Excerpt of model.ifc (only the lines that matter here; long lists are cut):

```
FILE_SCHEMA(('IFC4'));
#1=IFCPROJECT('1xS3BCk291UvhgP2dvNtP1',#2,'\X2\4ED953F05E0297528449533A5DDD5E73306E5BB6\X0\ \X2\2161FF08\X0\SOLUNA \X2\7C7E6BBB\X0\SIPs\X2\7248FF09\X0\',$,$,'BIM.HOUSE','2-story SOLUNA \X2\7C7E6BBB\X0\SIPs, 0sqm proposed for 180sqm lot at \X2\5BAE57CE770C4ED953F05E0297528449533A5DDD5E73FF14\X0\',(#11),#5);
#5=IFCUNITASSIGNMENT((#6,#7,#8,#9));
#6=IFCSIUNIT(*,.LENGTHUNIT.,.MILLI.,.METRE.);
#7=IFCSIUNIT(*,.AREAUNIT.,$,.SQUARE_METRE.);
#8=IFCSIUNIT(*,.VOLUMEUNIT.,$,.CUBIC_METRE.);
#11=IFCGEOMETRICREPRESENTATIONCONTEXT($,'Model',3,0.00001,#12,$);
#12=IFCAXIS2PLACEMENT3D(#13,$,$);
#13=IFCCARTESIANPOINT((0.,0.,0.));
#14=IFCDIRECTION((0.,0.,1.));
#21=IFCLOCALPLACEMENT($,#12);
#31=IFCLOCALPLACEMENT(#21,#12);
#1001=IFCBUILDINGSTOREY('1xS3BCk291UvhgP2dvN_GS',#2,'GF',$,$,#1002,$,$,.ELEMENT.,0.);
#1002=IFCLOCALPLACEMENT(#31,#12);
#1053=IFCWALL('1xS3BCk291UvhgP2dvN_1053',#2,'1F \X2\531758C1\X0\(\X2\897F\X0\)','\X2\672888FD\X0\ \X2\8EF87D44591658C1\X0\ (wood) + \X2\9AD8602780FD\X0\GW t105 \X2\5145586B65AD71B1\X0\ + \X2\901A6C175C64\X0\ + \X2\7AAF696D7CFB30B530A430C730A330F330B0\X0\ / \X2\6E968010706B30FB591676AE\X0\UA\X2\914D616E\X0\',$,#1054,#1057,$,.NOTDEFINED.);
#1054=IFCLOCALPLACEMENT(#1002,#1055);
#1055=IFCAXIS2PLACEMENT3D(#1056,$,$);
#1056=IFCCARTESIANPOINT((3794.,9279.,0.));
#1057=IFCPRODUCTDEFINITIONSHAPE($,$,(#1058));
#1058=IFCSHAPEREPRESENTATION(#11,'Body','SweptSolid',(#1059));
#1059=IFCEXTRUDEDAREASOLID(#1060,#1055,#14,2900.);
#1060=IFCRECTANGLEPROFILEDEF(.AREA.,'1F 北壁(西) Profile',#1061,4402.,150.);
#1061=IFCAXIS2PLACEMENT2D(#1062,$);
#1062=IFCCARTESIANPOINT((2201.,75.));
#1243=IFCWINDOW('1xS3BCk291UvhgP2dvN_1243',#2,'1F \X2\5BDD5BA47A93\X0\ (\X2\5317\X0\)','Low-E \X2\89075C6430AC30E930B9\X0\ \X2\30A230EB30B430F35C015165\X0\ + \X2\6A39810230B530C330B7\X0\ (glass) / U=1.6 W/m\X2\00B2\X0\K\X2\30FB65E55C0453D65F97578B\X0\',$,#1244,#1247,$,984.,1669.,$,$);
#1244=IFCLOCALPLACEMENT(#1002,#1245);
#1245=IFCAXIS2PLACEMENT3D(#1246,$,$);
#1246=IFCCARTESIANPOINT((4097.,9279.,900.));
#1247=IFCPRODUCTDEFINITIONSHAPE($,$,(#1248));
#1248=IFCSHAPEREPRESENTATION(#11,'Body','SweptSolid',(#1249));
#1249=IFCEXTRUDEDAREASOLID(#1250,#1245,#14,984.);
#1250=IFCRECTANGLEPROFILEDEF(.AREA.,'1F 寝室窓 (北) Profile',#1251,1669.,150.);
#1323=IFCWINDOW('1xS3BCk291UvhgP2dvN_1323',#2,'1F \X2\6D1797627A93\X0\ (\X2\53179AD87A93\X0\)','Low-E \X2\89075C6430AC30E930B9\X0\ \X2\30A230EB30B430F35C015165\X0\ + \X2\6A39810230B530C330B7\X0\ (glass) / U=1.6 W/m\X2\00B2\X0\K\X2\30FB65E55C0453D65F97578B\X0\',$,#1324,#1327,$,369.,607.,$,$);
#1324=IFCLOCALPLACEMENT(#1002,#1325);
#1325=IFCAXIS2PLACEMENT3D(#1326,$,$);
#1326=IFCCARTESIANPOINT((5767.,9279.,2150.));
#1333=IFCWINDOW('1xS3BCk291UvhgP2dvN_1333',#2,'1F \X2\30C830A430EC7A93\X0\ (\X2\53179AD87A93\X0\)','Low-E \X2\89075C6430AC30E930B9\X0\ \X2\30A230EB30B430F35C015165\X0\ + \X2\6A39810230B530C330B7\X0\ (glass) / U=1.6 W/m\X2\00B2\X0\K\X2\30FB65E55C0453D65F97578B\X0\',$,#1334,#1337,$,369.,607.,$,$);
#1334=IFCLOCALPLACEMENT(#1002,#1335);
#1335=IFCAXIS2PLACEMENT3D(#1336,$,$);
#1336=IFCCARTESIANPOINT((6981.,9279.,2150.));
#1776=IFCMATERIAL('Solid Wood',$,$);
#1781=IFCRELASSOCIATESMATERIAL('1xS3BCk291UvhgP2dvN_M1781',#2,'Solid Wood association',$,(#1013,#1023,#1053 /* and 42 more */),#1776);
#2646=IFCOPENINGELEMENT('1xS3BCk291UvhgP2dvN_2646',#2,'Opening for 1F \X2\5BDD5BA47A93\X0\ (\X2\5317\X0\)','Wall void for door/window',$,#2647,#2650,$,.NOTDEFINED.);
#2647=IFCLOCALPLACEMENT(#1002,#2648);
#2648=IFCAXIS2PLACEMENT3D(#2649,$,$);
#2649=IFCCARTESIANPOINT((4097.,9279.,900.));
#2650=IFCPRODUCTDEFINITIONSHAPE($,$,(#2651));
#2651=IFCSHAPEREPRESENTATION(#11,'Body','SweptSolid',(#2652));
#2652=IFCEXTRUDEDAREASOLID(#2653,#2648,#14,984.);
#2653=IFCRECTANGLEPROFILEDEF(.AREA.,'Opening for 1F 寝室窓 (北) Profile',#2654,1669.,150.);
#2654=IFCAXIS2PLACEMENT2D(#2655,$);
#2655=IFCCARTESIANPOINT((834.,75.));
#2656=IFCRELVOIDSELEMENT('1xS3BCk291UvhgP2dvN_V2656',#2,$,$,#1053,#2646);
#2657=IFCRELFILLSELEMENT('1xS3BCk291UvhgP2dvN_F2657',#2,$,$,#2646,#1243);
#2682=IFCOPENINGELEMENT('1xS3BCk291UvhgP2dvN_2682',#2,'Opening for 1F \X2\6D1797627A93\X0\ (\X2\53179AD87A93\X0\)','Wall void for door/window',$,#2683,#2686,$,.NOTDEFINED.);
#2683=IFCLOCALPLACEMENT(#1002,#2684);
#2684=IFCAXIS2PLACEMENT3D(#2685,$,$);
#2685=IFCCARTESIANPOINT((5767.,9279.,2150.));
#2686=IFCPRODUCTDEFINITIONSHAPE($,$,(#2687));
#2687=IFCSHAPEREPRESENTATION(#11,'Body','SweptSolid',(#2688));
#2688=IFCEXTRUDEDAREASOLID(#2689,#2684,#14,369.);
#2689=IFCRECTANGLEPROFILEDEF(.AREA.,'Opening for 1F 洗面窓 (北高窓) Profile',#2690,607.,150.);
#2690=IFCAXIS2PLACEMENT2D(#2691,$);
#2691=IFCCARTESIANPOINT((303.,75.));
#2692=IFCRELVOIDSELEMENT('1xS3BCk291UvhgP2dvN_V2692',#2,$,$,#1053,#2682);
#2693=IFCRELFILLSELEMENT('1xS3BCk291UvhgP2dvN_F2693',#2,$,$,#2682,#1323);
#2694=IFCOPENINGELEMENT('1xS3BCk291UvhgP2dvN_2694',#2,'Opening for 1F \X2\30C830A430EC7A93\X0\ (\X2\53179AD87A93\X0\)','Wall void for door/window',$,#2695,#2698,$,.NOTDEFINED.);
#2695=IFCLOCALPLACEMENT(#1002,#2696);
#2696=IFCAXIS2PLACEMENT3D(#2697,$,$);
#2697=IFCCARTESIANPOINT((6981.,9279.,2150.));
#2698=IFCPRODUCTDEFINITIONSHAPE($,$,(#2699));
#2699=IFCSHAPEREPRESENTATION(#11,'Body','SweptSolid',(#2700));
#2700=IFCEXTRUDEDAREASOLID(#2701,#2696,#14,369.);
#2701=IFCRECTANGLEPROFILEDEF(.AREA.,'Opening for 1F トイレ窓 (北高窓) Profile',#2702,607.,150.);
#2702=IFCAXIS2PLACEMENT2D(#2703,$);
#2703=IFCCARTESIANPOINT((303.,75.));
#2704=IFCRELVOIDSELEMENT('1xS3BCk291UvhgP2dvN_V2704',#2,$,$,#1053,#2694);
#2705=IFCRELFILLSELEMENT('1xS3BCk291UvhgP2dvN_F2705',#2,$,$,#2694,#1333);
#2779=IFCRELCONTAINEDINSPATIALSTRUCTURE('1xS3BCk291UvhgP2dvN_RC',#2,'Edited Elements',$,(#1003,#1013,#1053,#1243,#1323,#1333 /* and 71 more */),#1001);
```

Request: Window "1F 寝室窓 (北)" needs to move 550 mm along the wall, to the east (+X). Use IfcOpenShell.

```python
import ifcopenshell
import ifcopenshell.api.geometry
import ifcopenshell.util.placement

model = ifcopenshell.open("model.ifc")

window = model.by_id(1243)
opening = window.FillsVoids[0].RelatingOpeningElement
wall = opening.VoidsElements[0].RelatingBuildingElement

wall_matrix = ifcopenshell.util.placement.get_local_placement(wall.ObjectPlacement)
shift = wall_matrix[:3, 0] * 550.0
before = ifcopenshell.util.placement.get_local_placement(window.ObjectPlacement)[:3, 3].copy()

# The window is not placed relative to its opening, so move both.
for product in (opening, window):
    matrix = ifcopenshell.util.placement.get_local_placement(product.ObjectPlacement)
    matrix[:3, 3] += shift
    ifcopenshell.api.geometry.edit_object_placement(model, product=product, matrix=matrix, is_si=False)

after = ifcopenshell.util.placement.get_local_placement(window.ObjectPlacement)[:3, 3]
print("window moved by", (after - before).round(3) + 0.0)

model.write("model_edited.ifc")
```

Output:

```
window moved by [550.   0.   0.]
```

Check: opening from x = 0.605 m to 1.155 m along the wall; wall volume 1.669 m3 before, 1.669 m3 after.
